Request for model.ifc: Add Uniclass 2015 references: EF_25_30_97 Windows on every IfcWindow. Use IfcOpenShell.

First a look at what the model holds.

```python
import ifcopenshell

model = ifcopenshell.open("model.ifc")
print(model.schema)
print("classifications:", [c.Name for c in model.by_type("IfcClassification")])
for ifc_class in ("IfcDoor", "IfcRoof", "IfcStair", "IfcWall", "IfcWindow"):
    print(ifc_class, len(model.by_type(ifc_class)))
```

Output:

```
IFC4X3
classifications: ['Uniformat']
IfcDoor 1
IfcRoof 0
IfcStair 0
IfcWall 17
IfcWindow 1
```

```python
import ifcopenshell
import ifcopenshell.api.classification

model = ifcopenshell.open("model.ifc")

system = ifcopenshell.api.classification.add_classification(model, classification="Uniclass 2015")

codes = {
    "IfcWindow": ("EF_25_30_97", "Windows"),
}
for ifc_class, (code, name) in codes.items():
    products = model.by_type(ifc_class)
    ifcopenshell.api.classification.add_reference(
        model, products=products, classification=system, identification=code, name=name
    )
    print(code, len(products))

model.write("model_rev.ifc")
```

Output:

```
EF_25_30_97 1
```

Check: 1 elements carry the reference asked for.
